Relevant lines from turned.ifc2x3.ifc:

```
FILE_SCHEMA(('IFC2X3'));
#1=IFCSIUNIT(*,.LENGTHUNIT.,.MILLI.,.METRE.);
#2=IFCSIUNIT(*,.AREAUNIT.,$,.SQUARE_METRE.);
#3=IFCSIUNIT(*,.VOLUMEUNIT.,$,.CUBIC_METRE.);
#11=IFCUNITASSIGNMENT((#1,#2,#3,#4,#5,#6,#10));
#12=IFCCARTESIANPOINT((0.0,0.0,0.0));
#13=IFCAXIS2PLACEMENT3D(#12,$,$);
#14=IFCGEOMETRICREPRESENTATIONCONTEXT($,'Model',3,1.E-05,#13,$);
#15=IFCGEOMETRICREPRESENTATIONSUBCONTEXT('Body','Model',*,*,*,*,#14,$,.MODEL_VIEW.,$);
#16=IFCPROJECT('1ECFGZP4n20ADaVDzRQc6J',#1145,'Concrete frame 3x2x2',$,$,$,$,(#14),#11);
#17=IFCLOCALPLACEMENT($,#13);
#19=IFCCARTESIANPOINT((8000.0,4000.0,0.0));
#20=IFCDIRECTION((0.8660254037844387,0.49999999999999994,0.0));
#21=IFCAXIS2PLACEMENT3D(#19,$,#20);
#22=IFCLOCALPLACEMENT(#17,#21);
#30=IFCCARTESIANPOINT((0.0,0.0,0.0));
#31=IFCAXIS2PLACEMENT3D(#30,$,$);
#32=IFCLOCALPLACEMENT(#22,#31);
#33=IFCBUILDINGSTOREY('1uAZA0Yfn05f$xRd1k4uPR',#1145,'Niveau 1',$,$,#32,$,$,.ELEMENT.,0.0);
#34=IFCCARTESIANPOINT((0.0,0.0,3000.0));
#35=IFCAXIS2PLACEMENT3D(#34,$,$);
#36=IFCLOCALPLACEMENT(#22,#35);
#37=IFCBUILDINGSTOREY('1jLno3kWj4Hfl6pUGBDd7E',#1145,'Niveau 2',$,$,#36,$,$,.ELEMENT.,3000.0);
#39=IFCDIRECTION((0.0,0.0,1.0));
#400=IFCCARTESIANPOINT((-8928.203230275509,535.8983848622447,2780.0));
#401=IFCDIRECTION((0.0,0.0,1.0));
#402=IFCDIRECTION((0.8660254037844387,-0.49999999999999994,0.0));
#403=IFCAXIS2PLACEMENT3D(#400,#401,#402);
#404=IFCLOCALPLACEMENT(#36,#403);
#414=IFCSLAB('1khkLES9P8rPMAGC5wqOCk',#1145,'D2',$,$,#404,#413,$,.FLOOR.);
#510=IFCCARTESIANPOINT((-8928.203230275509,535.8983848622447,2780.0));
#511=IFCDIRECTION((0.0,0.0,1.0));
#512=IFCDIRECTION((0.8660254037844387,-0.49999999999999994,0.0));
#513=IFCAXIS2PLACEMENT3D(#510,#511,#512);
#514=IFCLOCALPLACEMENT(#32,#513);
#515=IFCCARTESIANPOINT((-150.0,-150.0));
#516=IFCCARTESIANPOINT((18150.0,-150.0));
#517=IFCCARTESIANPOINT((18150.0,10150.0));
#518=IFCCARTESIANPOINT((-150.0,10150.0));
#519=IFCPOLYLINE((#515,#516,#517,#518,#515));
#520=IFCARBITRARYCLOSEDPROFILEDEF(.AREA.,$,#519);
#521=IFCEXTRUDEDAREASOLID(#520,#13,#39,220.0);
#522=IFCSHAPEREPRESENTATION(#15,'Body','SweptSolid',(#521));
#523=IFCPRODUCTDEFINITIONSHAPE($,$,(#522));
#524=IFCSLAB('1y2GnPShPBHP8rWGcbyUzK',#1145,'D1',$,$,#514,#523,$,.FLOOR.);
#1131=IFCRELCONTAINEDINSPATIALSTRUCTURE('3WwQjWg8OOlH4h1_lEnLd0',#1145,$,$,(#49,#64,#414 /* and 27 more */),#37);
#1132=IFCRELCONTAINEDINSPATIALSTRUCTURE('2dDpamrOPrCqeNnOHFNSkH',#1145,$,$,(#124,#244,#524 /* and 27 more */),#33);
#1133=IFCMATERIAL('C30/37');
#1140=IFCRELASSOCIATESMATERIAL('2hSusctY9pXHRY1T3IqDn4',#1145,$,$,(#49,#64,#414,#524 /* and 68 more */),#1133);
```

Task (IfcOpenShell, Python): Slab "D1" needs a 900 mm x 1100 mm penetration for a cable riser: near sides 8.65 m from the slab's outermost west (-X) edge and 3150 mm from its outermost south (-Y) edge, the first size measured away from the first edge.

```python
import numpy as np
import ifcopenshell
import ifcopenshell.api.feature
import ifcopenshell.api.geometry
import ifcopenshell.api.root
import ifcopenshell.geom
import ifcopenshell.util.placement
import ifcopenshell.util.representation
import ifcopenshell.util.shape
import ifcopenshell.util.unit

model = ifcopenshell.open("turned.ifc2x3.ifc")
unit_scale = ifcopenshell.util.unit.calculate_unit_scale(model)
settings = ifcopenshell.geom.settings()


def volume(element):
    """Net volume in cubic metres, openings subtracted."""
    shape = ifcopenshell.geom.create_shape(settings, element)
    return ifcopenshell.util.shape.get_volume(shape.geometry)


slab = model.by_guid("1y2GnPShPBHP8rWGcbyUzK")
before = volume(slab)

# Extent in the slab's own axes, in metres. The edges named are its -X and -Y sides.
slab_shape = ifcopenshell.geom.create_shape(settings, slab)
vertices = ifcopenshell.util.shape.get_vertices(slab_shape.geometry)
x_min, y_min, bottom = vertices.min(axis=0)
top = vertices[:, 2].max()

opening = ifcopenshell.api.root.create_entity(model, ifc_class="IfcOpeningElement", name="Cable riser opening")
context = ifcopenshell.util.representation.get_context(model, "Model", "Body", "MODEL_VIEW")
width, depth = 0.9, 1.1
outline = [(0.0, 0.0), (width, 0.0), (width, depth), (0.0, depth), (0.0, 0.0)]
# Overshoot both faces by 50 mm so the cut is clean.
shape = ifcopenshell.api.geometry.add_slab_representation(
    model, context=context, depth=top - bottom + 0.1, polyline=outline
)
ifcopenshell.api.geometry.assign_representation(model, product=opening, representation=shape)

matrix = ifcopenshell.util.placement.get_local_placement(slab.ObjectPlacement)
matrix[:, 3] = matrix @ np.append(np.array([x_min + 8.65, y_min + 3.15, bottom - 0.05]) / unit_scale, 1.0)
ifcopenshell.api.geometry.edit_object_placement(model, product=opening, matrix=matrix, is_si=False)
ifcopenshell.api.feature.add_feature(model, feature=opening, element=slab)

after = volume(slab)

print(f"slab volume {before:.3f} -> {after:.3f} m3")

model.write("turned.ifc2x3_rev.ifc")
```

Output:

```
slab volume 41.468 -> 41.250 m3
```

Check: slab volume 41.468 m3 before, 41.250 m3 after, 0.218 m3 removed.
